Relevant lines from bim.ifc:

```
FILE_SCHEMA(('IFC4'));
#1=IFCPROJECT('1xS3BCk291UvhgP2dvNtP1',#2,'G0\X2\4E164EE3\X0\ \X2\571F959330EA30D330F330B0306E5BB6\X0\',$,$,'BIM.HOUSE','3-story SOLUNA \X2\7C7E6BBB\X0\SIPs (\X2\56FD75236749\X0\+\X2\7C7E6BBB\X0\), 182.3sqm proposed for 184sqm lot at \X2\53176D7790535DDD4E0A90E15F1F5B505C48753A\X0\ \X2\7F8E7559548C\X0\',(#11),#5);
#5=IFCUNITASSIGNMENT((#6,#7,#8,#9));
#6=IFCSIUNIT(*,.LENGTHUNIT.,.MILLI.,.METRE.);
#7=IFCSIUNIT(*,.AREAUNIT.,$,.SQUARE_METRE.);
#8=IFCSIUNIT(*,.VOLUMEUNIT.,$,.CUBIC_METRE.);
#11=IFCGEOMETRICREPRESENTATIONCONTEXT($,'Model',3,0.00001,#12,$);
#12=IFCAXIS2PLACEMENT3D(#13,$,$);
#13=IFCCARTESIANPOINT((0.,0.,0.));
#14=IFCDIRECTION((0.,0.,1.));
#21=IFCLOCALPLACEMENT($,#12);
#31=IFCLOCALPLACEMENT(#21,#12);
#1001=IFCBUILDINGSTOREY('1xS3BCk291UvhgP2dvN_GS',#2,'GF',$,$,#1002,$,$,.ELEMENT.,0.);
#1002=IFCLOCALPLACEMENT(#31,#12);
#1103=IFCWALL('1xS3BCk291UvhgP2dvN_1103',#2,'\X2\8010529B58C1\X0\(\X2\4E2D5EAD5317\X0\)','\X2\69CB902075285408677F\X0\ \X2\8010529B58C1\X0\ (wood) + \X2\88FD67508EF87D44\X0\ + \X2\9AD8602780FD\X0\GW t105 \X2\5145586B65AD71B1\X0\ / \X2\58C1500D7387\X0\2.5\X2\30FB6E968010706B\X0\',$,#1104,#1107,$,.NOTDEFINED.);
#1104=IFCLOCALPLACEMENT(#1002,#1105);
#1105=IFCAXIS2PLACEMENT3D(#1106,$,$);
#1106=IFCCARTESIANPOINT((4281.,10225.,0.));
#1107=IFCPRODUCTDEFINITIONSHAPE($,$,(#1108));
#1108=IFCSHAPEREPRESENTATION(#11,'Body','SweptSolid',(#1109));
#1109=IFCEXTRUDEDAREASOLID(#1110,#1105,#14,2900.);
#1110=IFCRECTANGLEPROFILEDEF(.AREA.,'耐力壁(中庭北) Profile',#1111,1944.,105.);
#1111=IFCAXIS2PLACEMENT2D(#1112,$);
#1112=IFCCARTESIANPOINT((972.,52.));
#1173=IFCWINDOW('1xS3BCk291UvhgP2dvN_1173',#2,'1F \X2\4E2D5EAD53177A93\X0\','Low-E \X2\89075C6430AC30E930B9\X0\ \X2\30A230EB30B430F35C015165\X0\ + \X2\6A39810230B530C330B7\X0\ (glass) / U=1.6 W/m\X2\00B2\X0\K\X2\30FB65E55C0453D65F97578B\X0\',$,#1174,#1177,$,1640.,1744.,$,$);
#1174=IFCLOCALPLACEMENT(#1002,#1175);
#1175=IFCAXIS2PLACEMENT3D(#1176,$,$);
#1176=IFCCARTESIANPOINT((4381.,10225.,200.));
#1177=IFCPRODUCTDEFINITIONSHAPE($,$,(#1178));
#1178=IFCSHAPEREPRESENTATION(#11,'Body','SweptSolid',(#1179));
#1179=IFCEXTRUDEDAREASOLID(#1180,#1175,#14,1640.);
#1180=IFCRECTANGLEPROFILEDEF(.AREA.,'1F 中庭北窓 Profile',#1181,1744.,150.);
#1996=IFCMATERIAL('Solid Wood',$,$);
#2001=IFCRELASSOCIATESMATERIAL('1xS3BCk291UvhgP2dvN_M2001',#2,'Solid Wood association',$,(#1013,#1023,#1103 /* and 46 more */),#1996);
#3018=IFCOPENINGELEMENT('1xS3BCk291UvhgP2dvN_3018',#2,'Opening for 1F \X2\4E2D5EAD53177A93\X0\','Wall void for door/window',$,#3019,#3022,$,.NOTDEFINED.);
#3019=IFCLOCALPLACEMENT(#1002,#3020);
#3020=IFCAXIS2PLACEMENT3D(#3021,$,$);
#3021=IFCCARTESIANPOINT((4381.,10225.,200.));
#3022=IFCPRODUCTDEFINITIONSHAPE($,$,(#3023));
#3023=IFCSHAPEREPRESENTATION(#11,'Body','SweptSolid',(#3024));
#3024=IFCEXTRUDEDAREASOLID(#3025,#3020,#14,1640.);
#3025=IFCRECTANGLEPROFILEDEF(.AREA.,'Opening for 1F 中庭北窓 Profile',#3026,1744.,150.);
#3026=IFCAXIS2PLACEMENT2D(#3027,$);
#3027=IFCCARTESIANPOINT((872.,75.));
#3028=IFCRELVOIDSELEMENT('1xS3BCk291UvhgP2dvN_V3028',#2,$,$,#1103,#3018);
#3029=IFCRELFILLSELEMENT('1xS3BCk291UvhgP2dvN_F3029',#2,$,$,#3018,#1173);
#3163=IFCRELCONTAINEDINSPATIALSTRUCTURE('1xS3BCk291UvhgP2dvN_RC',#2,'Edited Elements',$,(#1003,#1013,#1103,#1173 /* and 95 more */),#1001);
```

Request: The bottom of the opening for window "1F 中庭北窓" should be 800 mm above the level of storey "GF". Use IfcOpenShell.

```python
import numpy as np
import ifcopenshell
import ifcopenshell.api.geometry
import ifcopenshell.geom
import ifcopenshell.util.element
import ifcopenshell.util.placement
import ifcopenshell.util.shape
import ifcopenshell.util.unit

model = ifcopenshell.open("bim.ifc")
unit_scale = ifcopenshell.util.unit.calculate_unit_scale(model)

window = model.by_id(1173)
opening = window.FillsVoids[0].RelatingOpeningElement
storey = ifcopenshell.util.element.get_container(window, ifc_class="IfcBuildingStorey")
level = ifcopenshell.util.placement.get_local_placement(storey.ObjectPlacement)[2, 3]

# The opening's origin need not be at the sill, so measure its lowest point.
shape = ifcopenshell.geom.create_shape(ifcopenshell.geom.settings(), opening)
bottom = ifcopenshell.util.shape.get_shape_bottom_elevation(shape, shape.geometry) / unit_scale
dz = level + 800.0 - bottom

shift = np.array([0.0, 0.0, dz])
# The window is not placed relative to its opening, so move both.
for product in (opening, window):
    matrix = ifcopenshell.util.placement.get_local_placement(product.ObjectPlacement)
    matrix[:3, 3] += shift
    ifcopenshell.api.geometry.edit_object_placement(model, product=product, matrix=matrix, is_si=False)

print(f"moved by {dz * unit_scale:+.3f} m")

model.write("bim-out.ifc")
```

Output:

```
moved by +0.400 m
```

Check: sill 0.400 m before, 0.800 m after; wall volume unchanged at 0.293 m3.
